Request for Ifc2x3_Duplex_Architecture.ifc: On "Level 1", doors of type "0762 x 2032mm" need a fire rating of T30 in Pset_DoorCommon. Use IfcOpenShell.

First a look at what the model holds.

```python
import ifcopenshell
import ifcopenshell.util.element

model = ifcopenshell.open("Ifc2x3_Duplex_Architecture.ifc")
print(model.schema)
storey = next(s for s in model.by_type("IfcBuildingStorey") if s.Name == "Level 1")
doors = [e for e in ifcopenshell.util.element.get_decomposition(storey) if e.is_a("IfcDoor")]
seen = {}
for e in doors:
    element_type = ifcopenshell.util.element.get_type(e)
    key = (element_type.Name if element_type != e and element_type else None, ifcopenshell.util.element.get_pset(e, "Pset_DoorCommon", "FireRating"))
    seen[key] = seen.get(key, 0) + 1
for (name, value), count in sorted(seen.items(), key=str):
    print(count, "x", name, "|", value)
```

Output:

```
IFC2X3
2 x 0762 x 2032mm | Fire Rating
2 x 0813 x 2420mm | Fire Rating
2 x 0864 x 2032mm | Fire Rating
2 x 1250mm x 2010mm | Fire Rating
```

```python
import ifcopenshell
import ifcopenshell.api.pset
import ifcopenshell.util.element

model = ifcopenshell.open("Ifc2x3_Duplex_Architecture.ifc")

storey = next(s for s in model.by_type("IfcBuildingStorey") if s.Name == "Level 1")
doors = [e for e in ifcopenshell.util.element.get_decomposition(storey) if e.is_a("IfcDoor")]

count = 0
for e in doors:
    element_type = ifcopenshell.util.element.get_type(e)
    if element_type in (None, e) or element_type.Name != "0762 x 2032mm":
        continue
    # add_pset returns the element's existing set when there is one.
    pset = ifcopenshell.api.pset.add_pset(model, product=e, name="Pset_DoorCommon")
    ifcopenshell.api.pset.edit_pset(model, pset=pset, properties={"FireRating": "T30"})
    count += 1

print(count, "doors updated")

model.write("Ifc2x3_Duplex_Architecture_edited.ifc")
```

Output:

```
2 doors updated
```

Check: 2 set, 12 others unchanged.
